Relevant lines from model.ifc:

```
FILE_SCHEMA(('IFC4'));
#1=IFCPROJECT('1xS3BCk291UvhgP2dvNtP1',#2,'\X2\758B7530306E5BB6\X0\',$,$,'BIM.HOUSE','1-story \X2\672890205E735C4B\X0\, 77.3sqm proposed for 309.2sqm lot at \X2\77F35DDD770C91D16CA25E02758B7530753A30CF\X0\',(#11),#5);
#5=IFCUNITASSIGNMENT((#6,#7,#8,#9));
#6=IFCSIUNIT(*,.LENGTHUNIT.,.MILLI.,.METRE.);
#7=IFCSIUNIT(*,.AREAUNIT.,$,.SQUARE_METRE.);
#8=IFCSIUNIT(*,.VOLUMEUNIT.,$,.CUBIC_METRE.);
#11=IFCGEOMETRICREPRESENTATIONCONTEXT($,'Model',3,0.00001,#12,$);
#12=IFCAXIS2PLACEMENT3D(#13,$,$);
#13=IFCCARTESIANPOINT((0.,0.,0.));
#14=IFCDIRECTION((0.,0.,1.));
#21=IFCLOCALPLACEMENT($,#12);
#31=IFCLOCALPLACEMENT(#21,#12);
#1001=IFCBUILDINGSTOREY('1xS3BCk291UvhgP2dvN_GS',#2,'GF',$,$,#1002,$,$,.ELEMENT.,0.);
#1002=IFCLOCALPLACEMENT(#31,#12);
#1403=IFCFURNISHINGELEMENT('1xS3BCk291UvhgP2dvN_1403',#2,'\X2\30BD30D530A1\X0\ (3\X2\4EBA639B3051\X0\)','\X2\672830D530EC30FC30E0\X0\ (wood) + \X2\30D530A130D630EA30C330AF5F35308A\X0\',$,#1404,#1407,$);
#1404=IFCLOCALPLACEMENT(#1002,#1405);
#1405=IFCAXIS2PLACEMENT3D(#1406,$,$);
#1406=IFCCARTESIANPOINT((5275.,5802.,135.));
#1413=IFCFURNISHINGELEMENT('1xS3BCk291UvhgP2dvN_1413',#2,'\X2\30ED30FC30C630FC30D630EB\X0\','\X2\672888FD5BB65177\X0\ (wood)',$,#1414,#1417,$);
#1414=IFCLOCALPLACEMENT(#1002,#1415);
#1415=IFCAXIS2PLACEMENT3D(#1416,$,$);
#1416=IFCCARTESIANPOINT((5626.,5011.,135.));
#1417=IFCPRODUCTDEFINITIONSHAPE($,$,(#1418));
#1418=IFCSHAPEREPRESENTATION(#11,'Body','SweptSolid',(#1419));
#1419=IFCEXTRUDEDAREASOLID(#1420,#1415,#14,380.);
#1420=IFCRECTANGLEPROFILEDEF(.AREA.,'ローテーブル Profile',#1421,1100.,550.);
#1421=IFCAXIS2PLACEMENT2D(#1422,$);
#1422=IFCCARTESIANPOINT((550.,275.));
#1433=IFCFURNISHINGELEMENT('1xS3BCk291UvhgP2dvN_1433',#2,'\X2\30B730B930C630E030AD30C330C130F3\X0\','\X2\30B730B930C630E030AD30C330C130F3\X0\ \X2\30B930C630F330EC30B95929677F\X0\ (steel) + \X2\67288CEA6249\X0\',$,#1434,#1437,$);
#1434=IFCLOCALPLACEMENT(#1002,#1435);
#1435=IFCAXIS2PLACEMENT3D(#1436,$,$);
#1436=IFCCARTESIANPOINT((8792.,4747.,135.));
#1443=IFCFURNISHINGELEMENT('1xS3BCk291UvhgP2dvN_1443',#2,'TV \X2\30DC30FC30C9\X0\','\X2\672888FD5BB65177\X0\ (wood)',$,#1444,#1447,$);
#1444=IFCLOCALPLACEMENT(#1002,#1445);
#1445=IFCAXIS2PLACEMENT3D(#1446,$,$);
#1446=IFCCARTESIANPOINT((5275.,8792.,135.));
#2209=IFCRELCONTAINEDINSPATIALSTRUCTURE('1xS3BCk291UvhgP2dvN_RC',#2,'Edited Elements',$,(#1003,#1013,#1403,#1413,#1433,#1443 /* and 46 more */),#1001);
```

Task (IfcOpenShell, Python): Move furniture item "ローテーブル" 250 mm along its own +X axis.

```python
import ifcopenshell
import ifcopenshell.api.geometry
import ifcopenshell.util.placement
import ifcopenshell.util.unit

model = ifcopenshell.open("model.ifc")
unit_scale = ifcopenshell.util.unit.calculate_unit_scale(model)

item = model.by_guid("1xS3BCk291UvhgP2dvN_1413")
matrix = ifcopenshell.util.placement.get_local_placement(item.ObjectPlacement)
matrix[:3, 3] += matrix[:3, 0] * 0.25 / unit_scale
ifcopenshell.api.geometry.edit_object_placement(model, product=item, matrix=matrix, is_si=False)

print(ifcopenshell.util.placement.get_local_placement(item.ObjectPlacement).round(3) + 0.0)

model.write("model_edited.ifc")
```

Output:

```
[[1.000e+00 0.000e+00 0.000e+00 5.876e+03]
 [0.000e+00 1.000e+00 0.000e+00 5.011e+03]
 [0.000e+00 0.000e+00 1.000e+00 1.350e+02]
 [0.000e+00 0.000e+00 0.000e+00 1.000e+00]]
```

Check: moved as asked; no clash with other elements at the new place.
